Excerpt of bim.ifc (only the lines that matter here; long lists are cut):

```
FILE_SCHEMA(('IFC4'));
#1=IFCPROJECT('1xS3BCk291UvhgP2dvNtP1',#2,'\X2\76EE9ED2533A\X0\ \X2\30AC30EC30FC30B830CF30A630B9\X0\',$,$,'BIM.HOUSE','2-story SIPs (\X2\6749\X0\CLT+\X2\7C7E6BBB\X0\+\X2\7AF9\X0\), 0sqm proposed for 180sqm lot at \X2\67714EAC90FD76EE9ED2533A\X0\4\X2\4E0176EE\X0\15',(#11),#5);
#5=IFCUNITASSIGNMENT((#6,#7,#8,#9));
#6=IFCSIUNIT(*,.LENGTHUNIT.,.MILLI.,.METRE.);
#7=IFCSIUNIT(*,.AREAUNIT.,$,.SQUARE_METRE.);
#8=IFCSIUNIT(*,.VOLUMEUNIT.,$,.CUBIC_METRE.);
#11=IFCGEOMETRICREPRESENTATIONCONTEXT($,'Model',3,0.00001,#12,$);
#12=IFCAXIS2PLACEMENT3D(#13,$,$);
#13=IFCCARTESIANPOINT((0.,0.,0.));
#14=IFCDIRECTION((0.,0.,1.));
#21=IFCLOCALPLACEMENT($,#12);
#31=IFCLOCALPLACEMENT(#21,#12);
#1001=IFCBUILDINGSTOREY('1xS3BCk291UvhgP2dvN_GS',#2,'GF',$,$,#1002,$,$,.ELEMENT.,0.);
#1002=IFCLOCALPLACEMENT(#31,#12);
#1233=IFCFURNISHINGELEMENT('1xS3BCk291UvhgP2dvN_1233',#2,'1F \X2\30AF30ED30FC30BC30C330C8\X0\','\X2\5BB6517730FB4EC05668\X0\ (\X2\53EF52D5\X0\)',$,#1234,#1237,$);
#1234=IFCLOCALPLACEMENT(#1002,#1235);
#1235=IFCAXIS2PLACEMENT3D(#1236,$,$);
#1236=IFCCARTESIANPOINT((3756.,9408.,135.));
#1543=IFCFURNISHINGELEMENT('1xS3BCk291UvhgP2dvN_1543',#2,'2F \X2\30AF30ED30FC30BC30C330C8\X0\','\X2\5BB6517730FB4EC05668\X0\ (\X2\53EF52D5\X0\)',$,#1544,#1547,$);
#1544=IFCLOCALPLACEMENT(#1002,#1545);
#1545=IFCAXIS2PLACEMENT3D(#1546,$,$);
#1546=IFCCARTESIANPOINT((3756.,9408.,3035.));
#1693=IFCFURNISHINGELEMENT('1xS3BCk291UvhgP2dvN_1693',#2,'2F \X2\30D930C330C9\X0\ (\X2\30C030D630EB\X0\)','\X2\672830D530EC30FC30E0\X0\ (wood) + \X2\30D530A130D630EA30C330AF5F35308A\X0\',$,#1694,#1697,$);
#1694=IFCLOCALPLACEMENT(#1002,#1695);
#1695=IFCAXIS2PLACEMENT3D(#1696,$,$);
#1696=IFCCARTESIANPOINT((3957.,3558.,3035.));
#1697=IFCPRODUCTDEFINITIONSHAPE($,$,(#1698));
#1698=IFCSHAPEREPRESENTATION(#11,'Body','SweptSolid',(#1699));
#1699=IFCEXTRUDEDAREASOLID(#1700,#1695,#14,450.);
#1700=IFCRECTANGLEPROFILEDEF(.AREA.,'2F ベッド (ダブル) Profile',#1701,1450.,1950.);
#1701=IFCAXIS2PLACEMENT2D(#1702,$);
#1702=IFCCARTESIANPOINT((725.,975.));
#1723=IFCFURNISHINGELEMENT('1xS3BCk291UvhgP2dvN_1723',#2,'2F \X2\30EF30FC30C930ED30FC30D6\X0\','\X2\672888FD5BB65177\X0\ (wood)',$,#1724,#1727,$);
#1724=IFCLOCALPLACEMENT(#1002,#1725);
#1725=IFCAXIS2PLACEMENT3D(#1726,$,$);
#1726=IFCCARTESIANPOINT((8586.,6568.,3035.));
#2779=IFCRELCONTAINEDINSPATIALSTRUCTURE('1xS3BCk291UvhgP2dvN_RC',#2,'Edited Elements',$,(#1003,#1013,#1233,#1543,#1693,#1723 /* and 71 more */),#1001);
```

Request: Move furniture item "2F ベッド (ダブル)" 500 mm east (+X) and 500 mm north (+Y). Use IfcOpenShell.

```python
import ifcopenshell
import ifcopenshell.api.geometry
import ifcopenshell.util.placement
import ifcopenshell.util.unit

model = ifcopenshell.open("bim.ifc")
unit_scale = ifcopenshell.util.unit.calculate_unit_scale(model)

item = model.by_guid("1xS3BCk291UvhgP2dvN_1693")
matrix = ifcopenshell.util.placement.get_local_placement(item.ObjectPlacement)
matrix[0, 3] += 0.5 / unit_scale
matrix[1, 3] += 0.5 / unit_scale
ifcopenshell.api.geometry.edit_object_placement(model, product=item, matrix=matrix, is_si=False)

print(ifcopenshell.util.placement.get_local_placement(item.ObjectPlacement).round(3) + 0.0)

model.write("bim-out.ifc")
```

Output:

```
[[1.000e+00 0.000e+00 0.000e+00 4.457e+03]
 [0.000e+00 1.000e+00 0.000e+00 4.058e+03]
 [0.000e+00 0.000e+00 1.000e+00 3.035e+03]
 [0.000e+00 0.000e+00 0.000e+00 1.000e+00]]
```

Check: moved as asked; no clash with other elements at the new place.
